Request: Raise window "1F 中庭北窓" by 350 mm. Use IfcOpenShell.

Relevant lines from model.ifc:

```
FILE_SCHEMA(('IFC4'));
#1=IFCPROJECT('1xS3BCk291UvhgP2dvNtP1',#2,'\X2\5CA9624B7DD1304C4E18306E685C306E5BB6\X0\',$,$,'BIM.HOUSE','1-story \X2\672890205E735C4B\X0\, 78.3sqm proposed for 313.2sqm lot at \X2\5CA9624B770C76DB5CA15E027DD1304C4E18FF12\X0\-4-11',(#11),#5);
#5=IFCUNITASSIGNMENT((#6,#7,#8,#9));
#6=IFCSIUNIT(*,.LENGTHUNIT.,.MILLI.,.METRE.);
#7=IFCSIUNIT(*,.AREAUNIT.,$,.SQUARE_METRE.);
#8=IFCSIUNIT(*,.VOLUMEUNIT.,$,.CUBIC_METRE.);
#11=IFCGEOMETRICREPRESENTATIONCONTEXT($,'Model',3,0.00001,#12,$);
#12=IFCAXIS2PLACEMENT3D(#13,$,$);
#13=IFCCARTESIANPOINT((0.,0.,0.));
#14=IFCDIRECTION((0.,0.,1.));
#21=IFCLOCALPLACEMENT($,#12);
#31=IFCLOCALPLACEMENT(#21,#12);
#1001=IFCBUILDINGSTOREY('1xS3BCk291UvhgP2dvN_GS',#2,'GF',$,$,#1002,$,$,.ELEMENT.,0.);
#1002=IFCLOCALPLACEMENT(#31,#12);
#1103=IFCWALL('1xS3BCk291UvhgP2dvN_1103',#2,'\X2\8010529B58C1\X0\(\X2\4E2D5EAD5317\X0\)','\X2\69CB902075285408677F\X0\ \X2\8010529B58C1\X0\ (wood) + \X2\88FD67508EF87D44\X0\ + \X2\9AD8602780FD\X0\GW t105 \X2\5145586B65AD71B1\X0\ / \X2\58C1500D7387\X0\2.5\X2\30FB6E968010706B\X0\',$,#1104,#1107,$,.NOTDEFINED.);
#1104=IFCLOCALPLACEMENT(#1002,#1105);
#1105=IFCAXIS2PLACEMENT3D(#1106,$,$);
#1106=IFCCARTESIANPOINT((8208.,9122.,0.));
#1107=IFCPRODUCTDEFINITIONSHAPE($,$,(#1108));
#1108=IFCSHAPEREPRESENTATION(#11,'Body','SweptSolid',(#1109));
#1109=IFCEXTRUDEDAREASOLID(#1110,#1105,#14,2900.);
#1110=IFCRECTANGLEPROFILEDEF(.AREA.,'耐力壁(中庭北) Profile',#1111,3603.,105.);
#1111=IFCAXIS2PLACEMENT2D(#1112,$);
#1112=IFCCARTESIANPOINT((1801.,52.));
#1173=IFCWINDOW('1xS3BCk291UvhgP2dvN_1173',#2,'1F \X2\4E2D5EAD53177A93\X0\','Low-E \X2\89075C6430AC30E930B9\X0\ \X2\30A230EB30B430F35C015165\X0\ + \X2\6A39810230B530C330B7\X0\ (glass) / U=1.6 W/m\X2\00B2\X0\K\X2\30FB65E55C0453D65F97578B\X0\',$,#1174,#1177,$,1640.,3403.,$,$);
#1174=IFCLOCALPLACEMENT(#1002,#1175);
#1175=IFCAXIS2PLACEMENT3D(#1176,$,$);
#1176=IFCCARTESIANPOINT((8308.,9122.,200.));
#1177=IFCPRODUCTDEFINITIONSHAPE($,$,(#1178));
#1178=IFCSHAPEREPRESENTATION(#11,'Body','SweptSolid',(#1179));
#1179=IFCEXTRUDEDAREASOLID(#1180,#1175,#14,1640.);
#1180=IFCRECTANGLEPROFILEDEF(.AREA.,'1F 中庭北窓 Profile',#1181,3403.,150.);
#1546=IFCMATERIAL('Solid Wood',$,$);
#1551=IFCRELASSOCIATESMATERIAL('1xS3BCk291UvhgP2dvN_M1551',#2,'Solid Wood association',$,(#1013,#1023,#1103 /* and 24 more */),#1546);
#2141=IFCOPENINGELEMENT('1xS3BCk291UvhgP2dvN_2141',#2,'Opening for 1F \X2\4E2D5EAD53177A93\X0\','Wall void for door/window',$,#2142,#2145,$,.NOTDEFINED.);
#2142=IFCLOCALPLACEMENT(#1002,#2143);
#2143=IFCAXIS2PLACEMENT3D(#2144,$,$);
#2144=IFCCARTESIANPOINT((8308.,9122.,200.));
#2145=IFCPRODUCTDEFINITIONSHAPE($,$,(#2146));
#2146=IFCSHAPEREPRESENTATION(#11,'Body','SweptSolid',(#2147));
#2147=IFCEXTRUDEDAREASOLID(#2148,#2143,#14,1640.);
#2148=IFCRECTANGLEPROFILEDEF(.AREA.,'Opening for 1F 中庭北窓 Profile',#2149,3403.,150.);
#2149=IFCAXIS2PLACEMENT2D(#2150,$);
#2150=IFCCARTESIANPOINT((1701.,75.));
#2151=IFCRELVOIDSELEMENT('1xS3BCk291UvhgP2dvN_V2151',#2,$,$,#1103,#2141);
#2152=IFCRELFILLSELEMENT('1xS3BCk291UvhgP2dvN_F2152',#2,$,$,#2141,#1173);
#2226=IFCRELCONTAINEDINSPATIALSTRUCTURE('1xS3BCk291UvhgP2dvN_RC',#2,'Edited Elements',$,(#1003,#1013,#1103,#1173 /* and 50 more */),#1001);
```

```python
import numpy as np
import ifcopenshell
import ifcopenshell.api.geometry
import ifcopenshell.util.placement
import ifcopenshell.util.unit

model = ifcopenshell.open("model.ifc")
unit_scale = ifcopenshell.util.unit.calculate_unit_scale(model)

window = model.by_guid("1xS3BCk291UvhgP2dvN_1173")
opening = window.FillsVoids[0].RelatingOpeningElement
dz = 0.35 / unit_scale

shift = np.array([0.0, 0.0, dz])
# The window is not placed relative to its opening, so move both.
for product in (opening, window):
    matrix = ifcopenshell.util.placement.get_local_placement(product.ObjectPlacement)
    matrix[:3, 3] += shift
    ifcopenshell.api.geometry.edit_object_placement(model, product=product, matrix=matrix, is_si=False)

print(f"moved by {dz * unit_scale:+.3f} m")

model.write("model_edited.ifc")
```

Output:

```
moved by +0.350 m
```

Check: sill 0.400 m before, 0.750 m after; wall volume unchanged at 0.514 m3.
